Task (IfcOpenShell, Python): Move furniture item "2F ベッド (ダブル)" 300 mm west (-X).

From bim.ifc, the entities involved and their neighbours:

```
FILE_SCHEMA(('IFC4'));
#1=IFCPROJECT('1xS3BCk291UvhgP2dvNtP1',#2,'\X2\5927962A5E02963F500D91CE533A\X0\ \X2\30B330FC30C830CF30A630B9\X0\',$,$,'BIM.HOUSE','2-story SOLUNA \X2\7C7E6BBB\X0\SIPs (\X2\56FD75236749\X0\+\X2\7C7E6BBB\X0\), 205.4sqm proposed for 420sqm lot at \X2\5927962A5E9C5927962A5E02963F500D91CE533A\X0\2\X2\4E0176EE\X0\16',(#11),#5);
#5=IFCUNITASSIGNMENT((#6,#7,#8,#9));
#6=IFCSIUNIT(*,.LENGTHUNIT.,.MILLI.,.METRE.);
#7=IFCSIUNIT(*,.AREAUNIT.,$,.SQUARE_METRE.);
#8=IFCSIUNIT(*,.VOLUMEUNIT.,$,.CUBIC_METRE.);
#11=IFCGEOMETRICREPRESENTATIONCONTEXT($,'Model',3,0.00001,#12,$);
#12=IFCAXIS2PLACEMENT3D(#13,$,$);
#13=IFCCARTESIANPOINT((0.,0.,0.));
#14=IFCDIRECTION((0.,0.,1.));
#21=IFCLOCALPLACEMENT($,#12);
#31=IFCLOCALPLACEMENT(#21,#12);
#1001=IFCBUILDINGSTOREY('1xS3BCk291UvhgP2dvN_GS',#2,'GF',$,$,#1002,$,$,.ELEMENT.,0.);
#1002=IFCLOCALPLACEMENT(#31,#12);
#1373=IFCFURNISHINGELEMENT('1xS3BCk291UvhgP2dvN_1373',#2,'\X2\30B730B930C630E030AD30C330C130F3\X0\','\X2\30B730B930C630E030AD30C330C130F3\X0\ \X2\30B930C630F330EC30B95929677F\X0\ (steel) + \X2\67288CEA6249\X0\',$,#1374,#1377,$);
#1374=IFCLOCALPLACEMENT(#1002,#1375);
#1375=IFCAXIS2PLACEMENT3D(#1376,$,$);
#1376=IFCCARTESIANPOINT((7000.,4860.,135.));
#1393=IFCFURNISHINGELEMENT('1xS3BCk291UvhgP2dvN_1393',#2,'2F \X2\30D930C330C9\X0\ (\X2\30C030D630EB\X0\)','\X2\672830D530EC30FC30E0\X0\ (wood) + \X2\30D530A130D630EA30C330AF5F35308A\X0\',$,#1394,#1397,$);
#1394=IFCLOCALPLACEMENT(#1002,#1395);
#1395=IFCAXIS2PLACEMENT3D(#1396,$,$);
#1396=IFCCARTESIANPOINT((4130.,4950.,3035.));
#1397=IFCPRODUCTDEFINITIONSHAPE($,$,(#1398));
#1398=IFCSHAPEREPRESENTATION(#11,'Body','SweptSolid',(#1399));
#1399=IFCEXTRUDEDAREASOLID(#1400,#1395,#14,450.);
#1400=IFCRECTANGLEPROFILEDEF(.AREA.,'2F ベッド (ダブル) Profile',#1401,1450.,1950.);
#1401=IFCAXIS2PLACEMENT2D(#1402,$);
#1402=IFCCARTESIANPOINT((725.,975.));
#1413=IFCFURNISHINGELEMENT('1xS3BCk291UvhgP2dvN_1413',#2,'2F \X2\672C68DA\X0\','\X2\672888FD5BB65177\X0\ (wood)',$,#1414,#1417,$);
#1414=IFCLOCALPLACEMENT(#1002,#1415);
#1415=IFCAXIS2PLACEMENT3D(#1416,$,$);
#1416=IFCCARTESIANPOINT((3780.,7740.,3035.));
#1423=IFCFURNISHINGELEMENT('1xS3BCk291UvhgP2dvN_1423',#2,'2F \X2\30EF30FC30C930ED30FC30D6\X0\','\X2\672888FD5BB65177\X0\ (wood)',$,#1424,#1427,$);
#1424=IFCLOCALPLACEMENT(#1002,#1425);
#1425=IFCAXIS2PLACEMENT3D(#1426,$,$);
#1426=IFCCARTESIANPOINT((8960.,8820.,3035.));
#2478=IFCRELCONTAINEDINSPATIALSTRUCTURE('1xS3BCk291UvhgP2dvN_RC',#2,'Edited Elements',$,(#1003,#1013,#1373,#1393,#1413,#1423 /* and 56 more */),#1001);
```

```python
import ifcopenshell
import ifcopenshell.api.geometry
import ifcopenshell.util.placement

model = ifcopenshell.open("bim.ifc")

item = model.by_guid("1xS3BCk291UvhgP2dvN_1393")
matrix = ifcopenshell.util.placement.get_local_placement(item.ObjectPlacement)
matrix[0, 3] -= 300.0
ifcopenshell.api.geometry.edit_object_placement(model, product=item, matrix=matrix, is_si=False)

print(ifcopenshell.util.placement.get_local_placement(item.ObjectPlacement).round(3) + 0.0)

model.write("bim_v2.ifc")
```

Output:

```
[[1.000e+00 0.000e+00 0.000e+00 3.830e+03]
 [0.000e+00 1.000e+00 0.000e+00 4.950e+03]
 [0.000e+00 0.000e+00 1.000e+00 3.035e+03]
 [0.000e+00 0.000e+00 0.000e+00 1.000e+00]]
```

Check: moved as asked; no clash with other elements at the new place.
